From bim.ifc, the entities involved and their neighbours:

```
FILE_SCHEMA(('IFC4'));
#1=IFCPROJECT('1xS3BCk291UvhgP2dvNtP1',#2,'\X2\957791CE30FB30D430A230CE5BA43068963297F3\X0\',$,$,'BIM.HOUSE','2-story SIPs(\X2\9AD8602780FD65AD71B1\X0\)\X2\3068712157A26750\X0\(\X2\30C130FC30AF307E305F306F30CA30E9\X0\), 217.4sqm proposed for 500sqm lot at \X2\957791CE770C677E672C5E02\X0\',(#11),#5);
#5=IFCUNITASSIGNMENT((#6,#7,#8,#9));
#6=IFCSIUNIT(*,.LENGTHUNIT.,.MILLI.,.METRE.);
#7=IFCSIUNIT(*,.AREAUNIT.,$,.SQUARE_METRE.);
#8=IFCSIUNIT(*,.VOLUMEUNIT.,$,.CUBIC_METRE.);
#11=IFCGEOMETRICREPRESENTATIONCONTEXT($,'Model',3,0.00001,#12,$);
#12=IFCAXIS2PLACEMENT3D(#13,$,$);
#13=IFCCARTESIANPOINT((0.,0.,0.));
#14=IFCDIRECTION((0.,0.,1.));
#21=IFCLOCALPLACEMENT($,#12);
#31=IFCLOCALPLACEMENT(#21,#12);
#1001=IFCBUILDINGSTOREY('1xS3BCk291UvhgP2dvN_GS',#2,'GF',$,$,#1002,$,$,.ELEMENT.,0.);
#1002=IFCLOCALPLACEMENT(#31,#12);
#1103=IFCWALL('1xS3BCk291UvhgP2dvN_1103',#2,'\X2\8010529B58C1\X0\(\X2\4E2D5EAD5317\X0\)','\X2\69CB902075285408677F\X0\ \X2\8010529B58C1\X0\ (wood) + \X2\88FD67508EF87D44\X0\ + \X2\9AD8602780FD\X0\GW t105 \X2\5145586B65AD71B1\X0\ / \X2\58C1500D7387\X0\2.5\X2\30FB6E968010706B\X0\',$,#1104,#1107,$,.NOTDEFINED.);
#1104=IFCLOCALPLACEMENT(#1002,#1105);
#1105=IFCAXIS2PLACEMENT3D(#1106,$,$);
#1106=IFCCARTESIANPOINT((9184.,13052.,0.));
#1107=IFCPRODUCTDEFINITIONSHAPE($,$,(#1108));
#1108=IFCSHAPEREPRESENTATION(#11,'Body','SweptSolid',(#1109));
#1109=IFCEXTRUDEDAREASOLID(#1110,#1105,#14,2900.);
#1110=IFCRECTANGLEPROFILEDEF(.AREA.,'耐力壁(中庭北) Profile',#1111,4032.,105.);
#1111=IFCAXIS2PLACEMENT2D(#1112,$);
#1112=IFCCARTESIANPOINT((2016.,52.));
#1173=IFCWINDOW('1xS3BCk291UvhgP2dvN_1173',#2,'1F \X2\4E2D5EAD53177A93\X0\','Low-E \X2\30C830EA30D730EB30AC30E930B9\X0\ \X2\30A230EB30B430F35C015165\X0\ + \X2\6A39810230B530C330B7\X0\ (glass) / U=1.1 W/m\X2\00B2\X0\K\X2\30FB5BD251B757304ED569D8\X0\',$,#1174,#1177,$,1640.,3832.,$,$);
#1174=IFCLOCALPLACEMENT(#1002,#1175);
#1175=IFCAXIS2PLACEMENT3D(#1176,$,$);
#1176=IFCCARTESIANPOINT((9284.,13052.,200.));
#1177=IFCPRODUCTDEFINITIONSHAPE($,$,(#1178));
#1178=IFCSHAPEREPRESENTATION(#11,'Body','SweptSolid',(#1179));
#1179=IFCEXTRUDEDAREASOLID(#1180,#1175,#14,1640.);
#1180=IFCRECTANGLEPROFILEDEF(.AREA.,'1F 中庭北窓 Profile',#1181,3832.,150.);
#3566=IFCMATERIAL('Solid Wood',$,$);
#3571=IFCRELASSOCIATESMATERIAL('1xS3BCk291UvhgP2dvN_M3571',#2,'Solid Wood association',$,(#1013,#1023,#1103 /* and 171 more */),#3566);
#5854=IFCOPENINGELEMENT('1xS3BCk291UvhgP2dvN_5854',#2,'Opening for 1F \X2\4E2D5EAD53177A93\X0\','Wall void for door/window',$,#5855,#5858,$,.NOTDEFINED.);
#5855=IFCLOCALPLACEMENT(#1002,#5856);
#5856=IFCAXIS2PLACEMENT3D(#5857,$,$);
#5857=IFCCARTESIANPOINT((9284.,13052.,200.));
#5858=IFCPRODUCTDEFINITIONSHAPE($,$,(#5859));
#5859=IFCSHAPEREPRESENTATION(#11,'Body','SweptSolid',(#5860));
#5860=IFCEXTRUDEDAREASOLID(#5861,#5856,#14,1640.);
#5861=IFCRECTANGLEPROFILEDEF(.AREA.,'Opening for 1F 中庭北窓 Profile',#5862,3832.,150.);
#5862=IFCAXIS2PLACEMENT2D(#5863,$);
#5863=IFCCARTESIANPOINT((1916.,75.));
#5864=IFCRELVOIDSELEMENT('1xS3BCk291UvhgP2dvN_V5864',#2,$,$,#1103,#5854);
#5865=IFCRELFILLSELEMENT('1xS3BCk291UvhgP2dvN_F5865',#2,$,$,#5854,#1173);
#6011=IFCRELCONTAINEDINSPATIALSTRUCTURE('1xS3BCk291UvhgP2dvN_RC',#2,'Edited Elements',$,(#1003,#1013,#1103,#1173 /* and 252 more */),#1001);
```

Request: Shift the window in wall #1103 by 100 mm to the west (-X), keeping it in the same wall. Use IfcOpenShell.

```python
import ifcopenshell
import ifcopenshell.api.geometry
import ifcopenshell.util.placement

model = ifcopenshell.open("bim.ifc")

window = model.by_guid("1xS3BCk291UvhgP2dvN_1173")
opening = window.FillsVoids[0].RelatingOpeningElement
wall = opening.VoidsElements[0].RelatingBuildingElement

wall_matrix = ifcopenshell.util.placement.get_local_placement(wall.ObjectPlacement)
shift = wall_matrix[:3, 0] * -100.0
before = ifcopenshell.util.placement.get_local_placement(window.ObjectPlacement)[:3, 3].copy()

# The window is not placed relative to its opening, so move both.
for product in (opening, window):
    matrix = ifcopenshell.util.placement.get_local_placement(product.ObjectPlacement)
    matrix[:3, 3] += shift
    ifcopenshell.api.geometry.edit_object_placement(model, product=product, matrix=matrix, is_si=False)

after = ifcopenshell.util.placement.get_local_placement(window.ObjectPlacement)[:3, 3]
print("window moved by", (after - before).round(3) + 0.0)

model.write("bim_v2.ifc")
```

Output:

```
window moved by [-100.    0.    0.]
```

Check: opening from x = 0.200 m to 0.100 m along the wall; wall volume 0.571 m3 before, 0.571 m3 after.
